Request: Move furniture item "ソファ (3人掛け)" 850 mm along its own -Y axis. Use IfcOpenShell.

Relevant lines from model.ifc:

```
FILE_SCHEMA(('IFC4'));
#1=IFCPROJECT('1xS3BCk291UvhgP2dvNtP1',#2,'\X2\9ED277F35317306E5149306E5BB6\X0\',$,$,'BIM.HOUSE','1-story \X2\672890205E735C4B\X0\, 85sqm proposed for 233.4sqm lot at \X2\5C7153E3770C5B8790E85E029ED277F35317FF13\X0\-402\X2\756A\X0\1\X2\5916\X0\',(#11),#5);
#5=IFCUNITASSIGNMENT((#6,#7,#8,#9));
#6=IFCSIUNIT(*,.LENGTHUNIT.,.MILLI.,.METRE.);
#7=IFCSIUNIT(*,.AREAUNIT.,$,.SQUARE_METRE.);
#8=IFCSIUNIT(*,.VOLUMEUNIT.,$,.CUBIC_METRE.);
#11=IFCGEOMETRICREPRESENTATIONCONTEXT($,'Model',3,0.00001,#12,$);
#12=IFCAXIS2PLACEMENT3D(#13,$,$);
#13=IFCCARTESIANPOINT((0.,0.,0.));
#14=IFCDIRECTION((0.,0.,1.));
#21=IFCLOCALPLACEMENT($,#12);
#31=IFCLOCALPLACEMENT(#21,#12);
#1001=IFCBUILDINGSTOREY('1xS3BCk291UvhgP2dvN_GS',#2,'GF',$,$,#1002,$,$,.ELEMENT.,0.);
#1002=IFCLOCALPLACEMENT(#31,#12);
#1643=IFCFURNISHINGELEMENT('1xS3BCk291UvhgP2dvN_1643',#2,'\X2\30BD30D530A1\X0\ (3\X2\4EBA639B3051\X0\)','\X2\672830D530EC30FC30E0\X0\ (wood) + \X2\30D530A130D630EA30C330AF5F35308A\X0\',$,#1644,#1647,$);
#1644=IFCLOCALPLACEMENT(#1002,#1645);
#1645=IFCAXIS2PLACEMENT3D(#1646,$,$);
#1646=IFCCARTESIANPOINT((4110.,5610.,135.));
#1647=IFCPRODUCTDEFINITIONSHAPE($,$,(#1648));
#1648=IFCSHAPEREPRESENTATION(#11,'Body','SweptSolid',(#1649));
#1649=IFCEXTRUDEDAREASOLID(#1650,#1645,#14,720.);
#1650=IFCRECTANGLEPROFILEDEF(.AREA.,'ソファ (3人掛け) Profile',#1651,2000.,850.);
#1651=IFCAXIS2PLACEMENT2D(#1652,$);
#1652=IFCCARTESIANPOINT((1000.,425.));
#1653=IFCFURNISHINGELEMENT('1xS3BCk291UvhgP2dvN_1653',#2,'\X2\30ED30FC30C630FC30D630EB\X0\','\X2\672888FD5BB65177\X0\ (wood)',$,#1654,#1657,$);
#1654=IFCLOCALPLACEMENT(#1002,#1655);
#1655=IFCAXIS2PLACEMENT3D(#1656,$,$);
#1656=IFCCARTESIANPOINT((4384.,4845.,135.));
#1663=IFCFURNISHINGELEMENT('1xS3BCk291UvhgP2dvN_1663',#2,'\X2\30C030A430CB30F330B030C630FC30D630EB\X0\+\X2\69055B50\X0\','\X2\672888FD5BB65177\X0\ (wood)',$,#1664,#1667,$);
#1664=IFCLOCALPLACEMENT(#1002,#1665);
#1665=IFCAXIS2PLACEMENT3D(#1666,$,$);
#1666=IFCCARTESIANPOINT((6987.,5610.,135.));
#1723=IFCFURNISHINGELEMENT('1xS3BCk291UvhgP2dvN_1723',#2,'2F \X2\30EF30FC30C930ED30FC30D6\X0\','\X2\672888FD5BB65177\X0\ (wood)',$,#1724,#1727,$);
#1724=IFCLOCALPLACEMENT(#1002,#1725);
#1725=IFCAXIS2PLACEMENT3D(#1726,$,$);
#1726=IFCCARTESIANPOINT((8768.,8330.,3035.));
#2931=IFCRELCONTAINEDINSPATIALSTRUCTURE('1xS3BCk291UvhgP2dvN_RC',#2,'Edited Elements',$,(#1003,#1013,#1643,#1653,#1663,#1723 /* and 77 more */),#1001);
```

```python
import ifcopenshell
import ifcopenshell.api.geometry
import ifcopenshell.util.placement
import ifcopenshell.util.unit

model = ifcopenshell.open("model.ifc")
unit_scale = ifcopenshell.util.unit.calculate_unit_scale(model)

item = model.by_id(1643)
matrix = ifcopenshell.util.placement.get_local_placement(item.ObjectPlacement)
matrix[:3, 3] -= matrix[:3, 1] * 0.85 / unit_scale
ifcopenshell.api.geometry.edit_object_placement(model, product=item, matrix=matrix, is_si=False)

print(ifcopenshell.util.placement.get_local_placement(item.ObjectPlacement).round(3) + 0.0)

model.write("model_edited.ifc")
```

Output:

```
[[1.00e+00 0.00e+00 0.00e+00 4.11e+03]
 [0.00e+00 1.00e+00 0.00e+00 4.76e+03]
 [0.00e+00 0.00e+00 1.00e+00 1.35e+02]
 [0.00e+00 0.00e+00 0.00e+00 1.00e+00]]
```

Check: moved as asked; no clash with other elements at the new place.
